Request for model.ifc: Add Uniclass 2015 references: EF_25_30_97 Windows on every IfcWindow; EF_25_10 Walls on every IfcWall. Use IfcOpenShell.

First a look at what the model holds.

```python
import ifcopenshell

model = ifcopenshell.open("model.ifc")
print(model.schema)
print("classifications:", [c.Name for c in model.by_type("IfcClassification")])
for ifc_class in ("IfcDoor", "IfcRoof", "IfcStair", "IfcWall", "IfcWindow"):
    print(ifc_class, len(model.by_type(ifc_class)))
```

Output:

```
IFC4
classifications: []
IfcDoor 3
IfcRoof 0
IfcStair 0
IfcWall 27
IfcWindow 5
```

```python
import ifcopenshell
import ifcopenshell.api.classification

model = ifcopenshell.open("model.ifc")

system = ifcopenshell.api.classification.add_classification(model, classification="Uniclass 2015")

codes = {
    "IfcWindow": ("EF_25_30_97", "Windows"),
    "IfcWall": ("EF_25_10", "Walls"),
}
for ifc_class, (code, name) in codes.items():
    products = model.by_type(ifc_class)
    ifcopenshell.api.classification.add_reference(
        model, products=products, classification=system, identification=code, name=name
    )
    print(code, len(products))

model.write("model_v2.ifc")
```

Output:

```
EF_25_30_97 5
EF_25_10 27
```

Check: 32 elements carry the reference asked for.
